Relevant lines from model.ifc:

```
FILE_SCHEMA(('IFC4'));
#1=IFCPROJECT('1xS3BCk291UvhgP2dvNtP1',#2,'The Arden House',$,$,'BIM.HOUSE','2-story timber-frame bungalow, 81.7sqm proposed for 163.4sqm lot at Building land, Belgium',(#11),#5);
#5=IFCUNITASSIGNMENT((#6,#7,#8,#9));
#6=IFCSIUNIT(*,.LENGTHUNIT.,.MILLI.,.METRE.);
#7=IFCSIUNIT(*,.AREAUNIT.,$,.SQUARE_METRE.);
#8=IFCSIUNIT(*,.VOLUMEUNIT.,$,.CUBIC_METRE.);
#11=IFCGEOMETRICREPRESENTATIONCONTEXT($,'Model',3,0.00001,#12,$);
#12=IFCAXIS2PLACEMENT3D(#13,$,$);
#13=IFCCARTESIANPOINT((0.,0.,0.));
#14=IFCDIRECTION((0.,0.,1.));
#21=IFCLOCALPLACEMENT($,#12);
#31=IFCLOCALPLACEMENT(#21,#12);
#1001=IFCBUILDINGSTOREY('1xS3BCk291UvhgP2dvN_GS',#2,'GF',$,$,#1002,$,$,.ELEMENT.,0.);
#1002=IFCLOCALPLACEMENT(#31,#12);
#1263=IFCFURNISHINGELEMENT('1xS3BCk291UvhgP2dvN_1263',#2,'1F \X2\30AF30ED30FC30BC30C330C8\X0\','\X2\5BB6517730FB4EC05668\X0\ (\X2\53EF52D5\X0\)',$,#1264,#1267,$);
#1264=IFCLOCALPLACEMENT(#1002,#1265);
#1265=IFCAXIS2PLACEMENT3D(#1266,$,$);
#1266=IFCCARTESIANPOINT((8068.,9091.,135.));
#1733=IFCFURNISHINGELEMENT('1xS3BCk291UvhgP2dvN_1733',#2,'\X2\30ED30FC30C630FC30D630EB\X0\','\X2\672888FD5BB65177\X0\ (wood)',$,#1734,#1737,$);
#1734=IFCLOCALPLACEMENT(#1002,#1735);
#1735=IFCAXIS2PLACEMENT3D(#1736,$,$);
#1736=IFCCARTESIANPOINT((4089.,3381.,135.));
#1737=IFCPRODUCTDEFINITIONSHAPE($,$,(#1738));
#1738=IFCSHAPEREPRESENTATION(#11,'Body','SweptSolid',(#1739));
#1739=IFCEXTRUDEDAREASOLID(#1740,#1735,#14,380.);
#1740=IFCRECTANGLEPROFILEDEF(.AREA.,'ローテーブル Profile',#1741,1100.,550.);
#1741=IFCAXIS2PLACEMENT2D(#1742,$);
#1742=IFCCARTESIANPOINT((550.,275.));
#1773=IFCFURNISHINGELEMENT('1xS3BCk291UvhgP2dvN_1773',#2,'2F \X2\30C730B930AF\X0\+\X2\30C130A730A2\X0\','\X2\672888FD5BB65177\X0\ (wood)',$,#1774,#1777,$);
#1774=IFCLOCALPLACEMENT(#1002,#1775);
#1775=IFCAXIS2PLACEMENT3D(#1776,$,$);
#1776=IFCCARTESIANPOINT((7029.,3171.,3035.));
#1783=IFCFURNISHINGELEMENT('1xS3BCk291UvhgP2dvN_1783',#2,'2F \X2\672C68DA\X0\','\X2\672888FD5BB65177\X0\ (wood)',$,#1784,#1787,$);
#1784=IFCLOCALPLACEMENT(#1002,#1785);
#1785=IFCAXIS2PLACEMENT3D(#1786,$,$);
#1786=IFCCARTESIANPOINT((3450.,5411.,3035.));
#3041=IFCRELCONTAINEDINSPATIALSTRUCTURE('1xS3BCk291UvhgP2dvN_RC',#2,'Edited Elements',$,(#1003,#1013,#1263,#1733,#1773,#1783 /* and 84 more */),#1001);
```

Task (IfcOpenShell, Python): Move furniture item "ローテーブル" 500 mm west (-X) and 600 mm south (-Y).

```python
import ifcopenshell
import ifcopenshell.api.geometry
import ifcopenshell.util.placement

model = ifcopenshell.open("model.ifc")

item = model.by_guid("1xS3BCk291UvhgP2dvN_1733")
matrix = ifcopenshell.util.placement.get_local_placement(item.ObjectPlacement)
matrix[0, 3] -= 500.0
matrix[1, 3] -= 600.0
ifcopenshell.api.geometry.edit_object_placement(model, product=item, matrix=matrix, is_si=False)

print(ifcopenshell.util.placement.get_local_placement(item.ObjectPlacement).round(3) + 0.0)

model.write("model_updated.ifc")
```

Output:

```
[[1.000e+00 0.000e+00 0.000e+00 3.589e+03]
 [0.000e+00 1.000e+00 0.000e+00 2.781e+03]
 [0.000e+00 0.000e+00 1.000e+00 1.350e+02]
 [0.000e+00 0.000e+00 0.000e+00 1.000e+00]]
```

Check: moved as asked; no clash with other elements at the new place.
